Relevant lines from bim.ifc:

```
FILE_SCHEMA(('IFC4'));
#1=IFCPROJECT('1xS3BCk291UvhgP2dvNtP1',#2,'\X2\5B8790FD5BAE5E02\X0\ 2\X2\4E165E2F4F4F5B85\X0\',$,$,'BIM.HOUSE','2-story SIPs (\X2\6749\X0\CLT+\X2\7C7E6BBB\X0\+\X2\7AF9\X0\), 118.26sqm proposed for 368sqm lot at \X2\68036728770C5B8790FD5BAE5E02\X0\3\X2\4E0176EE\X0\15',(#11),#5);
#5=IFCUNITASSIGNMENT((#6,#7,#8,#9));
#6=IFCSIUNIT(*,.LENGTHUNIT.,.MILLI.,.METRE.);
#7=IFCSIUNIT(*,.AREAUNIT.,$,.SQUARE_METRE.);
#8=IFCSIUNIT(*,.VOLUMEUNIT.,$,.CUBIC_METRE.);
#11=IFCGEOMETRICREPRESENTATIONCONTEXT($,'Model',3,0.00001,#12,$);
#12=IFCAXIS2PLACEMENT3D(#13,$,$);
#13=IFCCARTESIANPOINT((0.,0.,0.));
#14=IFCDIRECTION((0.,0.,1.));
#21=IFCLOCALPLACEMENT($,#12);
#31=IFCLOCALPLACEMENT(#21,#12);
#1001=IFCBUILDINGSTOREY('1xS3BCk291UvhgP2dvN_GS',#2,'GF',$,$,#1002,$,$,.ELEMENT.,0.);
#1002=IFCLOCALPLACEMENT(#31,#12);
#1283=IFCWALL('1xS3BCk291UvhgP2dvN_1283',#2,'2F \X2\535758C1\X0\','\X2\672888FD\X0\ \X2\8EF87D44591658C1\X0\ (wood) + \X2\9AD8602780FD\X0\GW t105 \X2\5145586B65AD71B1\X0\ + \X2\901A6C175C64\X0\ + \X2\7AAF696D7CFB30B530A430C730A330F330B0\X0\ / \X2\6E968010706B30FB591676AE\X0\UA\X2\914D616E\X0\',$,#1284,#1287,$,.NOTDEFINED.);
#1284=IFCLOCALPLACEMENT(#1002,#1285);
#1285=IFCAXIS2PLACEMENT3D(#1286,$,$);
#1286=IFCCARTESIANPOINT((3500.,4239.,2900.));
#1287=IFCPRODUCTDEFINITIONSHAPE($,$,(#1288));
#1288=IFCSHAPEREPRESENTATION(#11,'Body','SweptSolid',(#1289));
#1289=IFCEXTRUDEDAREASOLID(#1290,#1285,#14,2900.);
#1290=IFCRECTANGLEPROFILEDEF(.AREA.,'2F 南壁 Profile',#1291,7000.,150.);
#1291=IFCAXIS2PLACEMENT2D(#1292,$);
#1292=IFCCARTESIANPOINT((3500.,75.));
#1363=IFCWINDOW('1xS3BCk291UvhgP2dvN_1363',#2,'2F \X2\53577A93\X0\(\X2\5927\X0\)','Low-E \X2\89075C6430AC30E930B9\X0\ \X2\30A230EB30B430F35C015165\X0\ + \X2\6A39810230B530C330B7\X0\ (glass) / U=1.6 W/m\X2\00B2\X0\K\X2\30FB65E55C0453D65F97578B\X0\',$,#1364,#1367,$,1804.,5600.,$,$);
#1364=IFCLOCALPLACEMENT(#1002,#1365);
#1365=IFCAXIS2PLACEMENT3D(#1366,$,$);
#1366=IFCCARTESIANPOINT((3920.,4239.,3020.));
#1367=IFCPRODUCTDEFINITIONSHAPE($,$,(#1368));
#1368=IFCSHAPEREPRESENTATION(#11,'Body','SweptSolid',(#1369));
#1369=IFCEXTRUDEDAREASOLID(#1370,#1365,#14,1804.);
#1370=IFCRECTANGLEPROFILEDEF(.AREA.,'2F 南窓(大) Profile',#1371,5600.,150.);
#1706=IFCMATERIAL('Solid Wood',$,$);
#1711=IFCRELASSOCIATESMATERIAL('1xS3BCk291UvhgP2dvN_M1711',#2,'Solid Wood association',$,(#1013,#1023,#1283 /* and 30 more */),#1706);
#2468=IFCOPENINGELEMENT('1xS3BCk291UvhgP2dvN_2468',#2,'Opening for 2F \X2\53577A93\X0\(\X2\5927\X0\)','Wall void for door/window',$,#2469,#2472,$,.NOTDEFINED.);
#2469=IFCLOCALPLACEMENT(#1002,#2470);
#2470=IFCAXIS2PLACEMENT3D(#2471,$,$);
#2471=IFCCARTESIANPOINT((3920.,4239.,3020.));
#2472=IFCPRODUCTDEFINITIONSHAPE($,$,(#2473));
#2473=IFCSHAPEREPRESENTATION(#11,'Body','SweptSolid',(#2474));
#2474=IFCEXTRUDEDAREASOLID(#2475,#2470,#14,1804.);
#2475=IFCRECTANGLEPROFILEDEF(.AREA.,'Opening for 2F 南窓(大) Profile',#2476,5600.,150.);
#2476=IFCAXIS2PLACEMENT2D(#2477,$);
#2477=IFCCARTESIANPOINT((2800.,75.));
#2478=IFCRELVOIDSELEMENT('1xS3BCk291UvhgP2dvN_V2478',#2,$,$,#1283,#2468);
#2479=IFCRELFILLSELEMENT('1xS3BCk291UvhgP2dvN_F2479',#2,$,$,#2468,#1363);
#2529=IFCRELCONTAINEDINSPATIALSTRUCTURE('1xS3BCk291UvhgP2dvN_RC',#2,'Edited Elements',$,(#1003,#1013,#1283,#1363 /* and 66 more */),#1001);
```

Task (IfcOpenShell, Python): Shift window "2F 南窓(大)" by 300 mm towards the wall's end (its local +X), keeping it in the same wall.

```python
import ifcopenshell
import ifcopenshell.api.geometry
import ifcopenshell.util.placement
import ifcopenshell.util.unit

model = ifcopenshell.open("bim.ifc")
unit_scale = ifcopenshell.util.unit.calculate_unit_scale(model)

window = model.by_guid("1xS3BCk291UvhgP2dvN_1363")
opening = window.FillsVoids[0].RelatingOpeningElement
wall = opening.VoidsElements[0].RelatingBuildingElement

wall_matrix = ifcopenshell.util.placement.get_local_placement(wall.ObjectPlacement)
shift = wall_matrix[:3, 0] * 0.3 / unit_scale
before = ifcopenshell.util.placement.get_local_placement(window.ObjectPlacement)[:3, 3].copy()

# The window is not placed relative to its opening, so move both.
for product in (opening, window):
    matrix = ifcopenshell.util.placement.get_local_placement(product.ObjectPlacement)
    matrix[:3, 3] += shift
    ifcopenshell.api.geometry.edit_object_placement(model, product=product, matrix=matrix, is_si=False)

after = ifcopenshell.util.placement.get_local_placement(window.ObjectPlacement)[:3, 3]
print("window moved by", (after - before).round(3) + 0.0)

model.write("bim-out.ifc")
```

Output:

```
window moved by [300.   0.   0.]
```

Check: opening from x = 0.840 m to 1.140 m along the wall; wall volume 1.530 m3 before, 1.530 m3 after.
